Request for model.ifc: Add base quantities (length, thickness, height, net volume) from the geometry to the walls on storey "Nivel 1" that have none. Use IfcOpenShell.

First a look at what the model holds.

```python
import ifcopenshell
import ifcopenshell.util.element
import ifcopenshell.util.unit

model = ifcopenshell.open("model.ifc")
print(model.schema)
for unit_type in ("LENGTHUNIT", "AREAUNIT", "VOLUMEUNIT"):
    print(unit_type, ifcopenshell.util.unit.calculate_unit_scale(model, unit_type))
storey = next(s for s in model.by_type("IfcBuildingStorey") if s.Name == "Nivel 1")
walls = [e for e in ifcopenshell.util.element.get_decomposition(storey) if e.is_a("IfcWall")]
for e in sorted(walls, key=lambda e: e.id()):
    print(e.id(), e.is_a(), e.Name, list(ifcopenshell.util.element.get_psets(e, qtos_only=True)), sep=" | ")
```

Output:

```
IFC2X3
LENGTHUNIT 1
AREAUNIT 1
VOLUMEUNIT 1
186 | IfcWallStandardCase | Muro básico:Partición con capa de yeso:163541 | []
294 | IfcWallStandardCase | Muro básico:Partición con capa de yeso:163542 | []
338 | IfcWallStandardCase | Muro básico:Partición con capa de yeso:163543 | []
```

```python
import ifcopenshell
import ifcopenshell.api.pset
import ifcopenshell.geom
import ifcopenshell.util.element
import ifcopenshell.util.shape
import ifcopenshell.util.unit

model = ifcopenshell.open("model.ifc")
unit_scale = ifcopenshell.util.unit.calculate_unit_scale(model)
volume_scale = ifcopenshell.util.unit.calculate_unit_scale(model, "VOLUMEUNIT")
settings = ifcopenshell.geom.settings()

storey = next(s for s in model.by_type("IfcBuildingStorey") if s.Name == "Nivel 1")
walls = [e for e in ifcopenshell.util.element.get_decomposition(storey) if e.is_a("IfcWall")]

for e in sorted(walls, key=lambda e: e.id()):
    if ifcopenshell.util.element.get_psets(e, qtos_only=True, should_inherit=False):
        continue
    # Geometry comes back in metres, in the element's own axes.
    shape = ifcopenshell.geom.create_shape(settings, e)
    values = {
        "Length": ifcopenshell.util.shape.get_x(shape.geometry) / unit_scale,
        "Width": ifcopenshell.util.shape.get_y(shape.geometry) / unit_scale,
        "Height": ifcopenshell.util.shape.get_z(shape.geometry) / unit_scale,
        "NetVolume": ifcopenshell.util.shape.get_volume(shape.geometry) / volume_scale,
    }
    qto = ifcopenshell.api.pset.add_qto(model, product=e, name="BaseQuantities")
    ifcopenshell.api.pset.edit_qto(model, qto=qto, properties=values)
    print(e.id(), {k: round(v, 3) for k, v in values.items()})

model.write("model_v2.ifc")
```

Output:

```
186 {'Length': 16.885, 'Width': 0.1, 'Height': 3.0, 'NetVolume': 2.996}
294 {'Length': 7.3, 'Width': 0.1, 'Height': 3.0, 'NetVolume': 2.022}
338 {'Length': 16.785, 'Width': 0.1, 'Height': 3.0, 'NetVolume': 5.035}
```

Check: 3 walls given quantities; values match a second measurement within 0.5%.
